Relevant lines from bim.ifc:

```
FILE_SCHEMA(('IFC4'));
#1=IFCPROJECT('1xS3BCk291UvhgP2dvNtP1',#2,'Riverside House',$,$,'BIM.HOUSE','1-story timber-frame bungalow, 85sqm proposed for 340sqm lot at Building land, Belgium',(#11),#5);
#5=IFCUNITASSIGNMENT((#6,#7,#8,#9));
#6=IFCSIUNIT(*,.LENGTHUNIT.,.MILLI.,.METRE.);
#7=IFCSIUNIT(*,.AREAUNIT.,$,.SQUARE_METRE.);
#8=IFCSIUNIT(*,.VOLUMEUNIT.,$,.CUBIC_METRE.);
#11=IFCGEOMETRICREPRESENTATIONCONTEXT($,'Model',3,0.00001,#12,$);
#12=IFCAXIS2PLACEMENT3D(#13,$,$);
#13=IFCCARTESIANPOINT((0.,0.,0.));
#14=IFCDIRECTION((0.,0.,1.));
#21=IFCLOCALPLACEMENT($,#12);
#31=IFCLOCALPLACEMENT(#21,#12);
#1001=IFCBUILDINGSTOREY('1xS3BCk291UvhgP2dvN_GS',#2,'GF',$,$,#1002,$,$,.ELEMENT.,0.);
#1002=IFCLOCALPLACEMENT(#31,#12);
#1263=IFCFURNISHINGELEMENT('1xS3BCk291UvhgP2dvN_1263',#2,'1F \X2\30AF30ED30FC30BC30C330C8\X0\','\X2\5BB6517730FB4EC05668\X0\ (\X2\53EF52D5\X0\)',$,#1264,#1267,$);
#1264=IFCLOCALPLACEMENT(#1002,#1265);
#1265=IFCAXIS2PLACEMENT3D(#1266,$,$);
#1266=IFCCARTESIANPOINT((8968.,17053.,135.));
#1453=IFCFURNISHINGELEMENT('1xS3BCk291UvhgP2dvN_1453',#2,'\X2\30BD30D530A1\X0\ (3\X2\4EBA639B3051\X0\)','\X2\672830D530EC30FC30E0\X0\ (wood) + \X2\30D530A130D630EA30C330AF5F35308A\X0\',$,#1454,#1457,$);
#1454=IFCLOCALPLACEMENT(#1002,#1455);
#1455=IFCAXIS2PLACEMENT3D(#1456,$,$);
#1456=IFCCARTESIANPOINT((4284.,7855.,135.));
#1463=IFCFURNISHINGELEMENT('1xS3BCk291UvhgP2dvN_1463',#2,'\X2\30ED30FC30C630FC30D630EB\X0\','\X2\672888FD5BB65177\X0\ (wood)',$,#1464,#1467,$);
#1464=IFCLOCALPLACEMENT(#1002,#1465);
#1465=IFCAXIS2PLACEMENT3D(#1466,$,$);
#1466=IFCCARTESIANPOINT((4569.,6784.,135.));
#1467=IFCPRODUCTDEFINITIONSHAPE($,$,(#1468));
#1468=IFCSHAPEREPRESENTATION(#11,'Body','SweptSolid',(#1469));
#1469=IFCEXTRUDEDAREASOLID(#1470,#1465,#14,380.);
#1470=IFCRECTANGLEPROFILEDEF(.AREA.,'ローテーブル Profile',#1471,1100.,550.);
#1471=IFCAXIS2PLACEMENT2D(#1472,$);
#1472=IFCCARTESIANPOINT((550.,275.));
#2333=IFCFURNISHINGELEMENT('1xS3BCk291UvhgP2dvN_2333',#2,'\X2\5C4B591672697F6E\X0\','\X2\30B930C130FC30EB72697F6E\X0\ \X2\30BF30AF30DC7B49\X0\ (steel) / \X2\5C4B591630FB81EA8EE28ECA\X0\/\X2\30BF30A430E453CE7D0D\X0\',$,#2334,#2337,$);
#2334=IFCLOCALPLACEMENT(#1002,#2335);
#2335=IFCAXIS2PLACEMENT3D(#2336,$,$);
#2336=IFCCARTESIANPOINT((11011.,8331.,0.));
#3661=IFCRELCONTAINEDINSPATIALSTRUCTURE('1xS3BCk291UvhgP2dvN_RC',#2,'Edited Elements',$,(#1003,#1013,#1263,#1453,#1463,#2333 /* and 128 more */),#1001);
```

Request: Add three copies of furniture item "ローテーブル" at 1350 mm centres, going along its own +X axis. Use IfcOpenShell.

```python
import ifcopenshell
import ifcopenshell.api.geometry
import ifcopenshell.api.root
import ifcopenshell.util.element
import ifcopenshell.util.placement
import ifcopenshell.util.unit

model = ifcopenshell.open("bim.ifc")
unit_scale = ifcopenshell.util.unit.calculate_unit_scale(model)


def reuse_history(source, copy):
    """copy_class also copies each property set's owner history, people and application; keep the originals."""
    for rel in copy.IsDefinedBy:
        if rel.is_a("IfcRelDefinesByProperties") and (history := rel.RelatingPropertyDefinition.OwnerHistory):
            rel.RelatingPropertyDefinition.OwnerHistory = source.OwnerHistory
            ifcopenshell.util.element.remove_deep2(model, history)


source = model.by_guid("1xS3BCk291UvhgP2dvN_1463")
base = ifcopenshell.util.placement.get_local_placement(source.ObjectPlacement)
step = base[:3, 0] * 1.35 / unit_scale

for i in range(1, 4):
    copy = ifcopenshell.api.root.copy_class(model, product=source)
    copy.Representation = ifcopenshell.util.element.copy_deep(
        model, source.Representation, exclude=["IfcGeometricRepresentationContext", "IfcRepresentationMap"]
    )
    reuse_history(source, copy)
    matrix = base.copy()
    matrix[:3, 3] += i * step
    print("added at", matrix[:3, 3].round(3) + 0.0)
    ifcopenshell.api.geometry.edit_object_placement(model, product=copy, matrix=matrix, is_si=False)

model.write("bim_updated.ifc")
```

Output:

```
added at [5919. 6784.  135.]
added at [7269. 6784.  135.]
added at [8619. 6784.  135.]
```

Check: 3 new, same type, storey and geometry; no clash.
